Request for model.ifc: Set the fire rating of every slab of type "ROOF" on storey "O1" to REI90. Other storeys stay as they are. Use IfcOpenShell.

First a look at what the model holds.

```python
import ifcopenshell
import ifcopenshell.util.element

model = ifcopenshell.open("model.ifc")
print(model.schema)
storey = next(s for s in model.by_type("IfcBuildingStorey") if s.Name == "O1")
slabs = [e for e in ifcopenshell.util.element.get_decomposition(storey) if e.is_a("IfcSlab")]
seen = {}
for e in slabs:
    element_type = ifcopenshell.util.element.get_type(e)
    key = (element_type.Name if element_type != e and element_type else None, ifcopenshell.util.element.get_pset(e, "Pset_SlabCommon", "FireRating"))
    seen[key] = seen.get(key, 0) + 1
for (name, value), count in sorted(seen.items(), key=str):
    print(count, "x", name, "|", value)
```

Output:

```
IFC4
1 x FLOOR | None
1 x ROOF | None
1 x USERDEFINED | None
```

```python
import ifcopenshell
import ifcopenshell.api.pset
import ifcopenshell.util.element

model = ifcopenshell.open("model.ifc")

storey = next(s for s in model.by_type("IfcBuildingStorey") if s.Name == "O1")
slabs = [e for e in ifcopenshell.util.element.get_decomposition(storey) if e.is_a("IfcSlab")]

count = 0
for e in slabs:
    element_type = ifcopenshell.util.element.get_type(e)
    if element_type in (None, e) or element_type.Name != "ROOF":
        continue
    # add_pset returns the element's existing set when there is one.
    pset = ifcopenshell.api.pset.add_pset(model, product=e, name="Pset_SlabCommon")
    ifcopenshell.api.pset.edit_pset(model, pset=pset, properties={"FireRating": "REI90"})
    count += 1

print(count, "slabs updated")

model.write("model_rev.ifc")
```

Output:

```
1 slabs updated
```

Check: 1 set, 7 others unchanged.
